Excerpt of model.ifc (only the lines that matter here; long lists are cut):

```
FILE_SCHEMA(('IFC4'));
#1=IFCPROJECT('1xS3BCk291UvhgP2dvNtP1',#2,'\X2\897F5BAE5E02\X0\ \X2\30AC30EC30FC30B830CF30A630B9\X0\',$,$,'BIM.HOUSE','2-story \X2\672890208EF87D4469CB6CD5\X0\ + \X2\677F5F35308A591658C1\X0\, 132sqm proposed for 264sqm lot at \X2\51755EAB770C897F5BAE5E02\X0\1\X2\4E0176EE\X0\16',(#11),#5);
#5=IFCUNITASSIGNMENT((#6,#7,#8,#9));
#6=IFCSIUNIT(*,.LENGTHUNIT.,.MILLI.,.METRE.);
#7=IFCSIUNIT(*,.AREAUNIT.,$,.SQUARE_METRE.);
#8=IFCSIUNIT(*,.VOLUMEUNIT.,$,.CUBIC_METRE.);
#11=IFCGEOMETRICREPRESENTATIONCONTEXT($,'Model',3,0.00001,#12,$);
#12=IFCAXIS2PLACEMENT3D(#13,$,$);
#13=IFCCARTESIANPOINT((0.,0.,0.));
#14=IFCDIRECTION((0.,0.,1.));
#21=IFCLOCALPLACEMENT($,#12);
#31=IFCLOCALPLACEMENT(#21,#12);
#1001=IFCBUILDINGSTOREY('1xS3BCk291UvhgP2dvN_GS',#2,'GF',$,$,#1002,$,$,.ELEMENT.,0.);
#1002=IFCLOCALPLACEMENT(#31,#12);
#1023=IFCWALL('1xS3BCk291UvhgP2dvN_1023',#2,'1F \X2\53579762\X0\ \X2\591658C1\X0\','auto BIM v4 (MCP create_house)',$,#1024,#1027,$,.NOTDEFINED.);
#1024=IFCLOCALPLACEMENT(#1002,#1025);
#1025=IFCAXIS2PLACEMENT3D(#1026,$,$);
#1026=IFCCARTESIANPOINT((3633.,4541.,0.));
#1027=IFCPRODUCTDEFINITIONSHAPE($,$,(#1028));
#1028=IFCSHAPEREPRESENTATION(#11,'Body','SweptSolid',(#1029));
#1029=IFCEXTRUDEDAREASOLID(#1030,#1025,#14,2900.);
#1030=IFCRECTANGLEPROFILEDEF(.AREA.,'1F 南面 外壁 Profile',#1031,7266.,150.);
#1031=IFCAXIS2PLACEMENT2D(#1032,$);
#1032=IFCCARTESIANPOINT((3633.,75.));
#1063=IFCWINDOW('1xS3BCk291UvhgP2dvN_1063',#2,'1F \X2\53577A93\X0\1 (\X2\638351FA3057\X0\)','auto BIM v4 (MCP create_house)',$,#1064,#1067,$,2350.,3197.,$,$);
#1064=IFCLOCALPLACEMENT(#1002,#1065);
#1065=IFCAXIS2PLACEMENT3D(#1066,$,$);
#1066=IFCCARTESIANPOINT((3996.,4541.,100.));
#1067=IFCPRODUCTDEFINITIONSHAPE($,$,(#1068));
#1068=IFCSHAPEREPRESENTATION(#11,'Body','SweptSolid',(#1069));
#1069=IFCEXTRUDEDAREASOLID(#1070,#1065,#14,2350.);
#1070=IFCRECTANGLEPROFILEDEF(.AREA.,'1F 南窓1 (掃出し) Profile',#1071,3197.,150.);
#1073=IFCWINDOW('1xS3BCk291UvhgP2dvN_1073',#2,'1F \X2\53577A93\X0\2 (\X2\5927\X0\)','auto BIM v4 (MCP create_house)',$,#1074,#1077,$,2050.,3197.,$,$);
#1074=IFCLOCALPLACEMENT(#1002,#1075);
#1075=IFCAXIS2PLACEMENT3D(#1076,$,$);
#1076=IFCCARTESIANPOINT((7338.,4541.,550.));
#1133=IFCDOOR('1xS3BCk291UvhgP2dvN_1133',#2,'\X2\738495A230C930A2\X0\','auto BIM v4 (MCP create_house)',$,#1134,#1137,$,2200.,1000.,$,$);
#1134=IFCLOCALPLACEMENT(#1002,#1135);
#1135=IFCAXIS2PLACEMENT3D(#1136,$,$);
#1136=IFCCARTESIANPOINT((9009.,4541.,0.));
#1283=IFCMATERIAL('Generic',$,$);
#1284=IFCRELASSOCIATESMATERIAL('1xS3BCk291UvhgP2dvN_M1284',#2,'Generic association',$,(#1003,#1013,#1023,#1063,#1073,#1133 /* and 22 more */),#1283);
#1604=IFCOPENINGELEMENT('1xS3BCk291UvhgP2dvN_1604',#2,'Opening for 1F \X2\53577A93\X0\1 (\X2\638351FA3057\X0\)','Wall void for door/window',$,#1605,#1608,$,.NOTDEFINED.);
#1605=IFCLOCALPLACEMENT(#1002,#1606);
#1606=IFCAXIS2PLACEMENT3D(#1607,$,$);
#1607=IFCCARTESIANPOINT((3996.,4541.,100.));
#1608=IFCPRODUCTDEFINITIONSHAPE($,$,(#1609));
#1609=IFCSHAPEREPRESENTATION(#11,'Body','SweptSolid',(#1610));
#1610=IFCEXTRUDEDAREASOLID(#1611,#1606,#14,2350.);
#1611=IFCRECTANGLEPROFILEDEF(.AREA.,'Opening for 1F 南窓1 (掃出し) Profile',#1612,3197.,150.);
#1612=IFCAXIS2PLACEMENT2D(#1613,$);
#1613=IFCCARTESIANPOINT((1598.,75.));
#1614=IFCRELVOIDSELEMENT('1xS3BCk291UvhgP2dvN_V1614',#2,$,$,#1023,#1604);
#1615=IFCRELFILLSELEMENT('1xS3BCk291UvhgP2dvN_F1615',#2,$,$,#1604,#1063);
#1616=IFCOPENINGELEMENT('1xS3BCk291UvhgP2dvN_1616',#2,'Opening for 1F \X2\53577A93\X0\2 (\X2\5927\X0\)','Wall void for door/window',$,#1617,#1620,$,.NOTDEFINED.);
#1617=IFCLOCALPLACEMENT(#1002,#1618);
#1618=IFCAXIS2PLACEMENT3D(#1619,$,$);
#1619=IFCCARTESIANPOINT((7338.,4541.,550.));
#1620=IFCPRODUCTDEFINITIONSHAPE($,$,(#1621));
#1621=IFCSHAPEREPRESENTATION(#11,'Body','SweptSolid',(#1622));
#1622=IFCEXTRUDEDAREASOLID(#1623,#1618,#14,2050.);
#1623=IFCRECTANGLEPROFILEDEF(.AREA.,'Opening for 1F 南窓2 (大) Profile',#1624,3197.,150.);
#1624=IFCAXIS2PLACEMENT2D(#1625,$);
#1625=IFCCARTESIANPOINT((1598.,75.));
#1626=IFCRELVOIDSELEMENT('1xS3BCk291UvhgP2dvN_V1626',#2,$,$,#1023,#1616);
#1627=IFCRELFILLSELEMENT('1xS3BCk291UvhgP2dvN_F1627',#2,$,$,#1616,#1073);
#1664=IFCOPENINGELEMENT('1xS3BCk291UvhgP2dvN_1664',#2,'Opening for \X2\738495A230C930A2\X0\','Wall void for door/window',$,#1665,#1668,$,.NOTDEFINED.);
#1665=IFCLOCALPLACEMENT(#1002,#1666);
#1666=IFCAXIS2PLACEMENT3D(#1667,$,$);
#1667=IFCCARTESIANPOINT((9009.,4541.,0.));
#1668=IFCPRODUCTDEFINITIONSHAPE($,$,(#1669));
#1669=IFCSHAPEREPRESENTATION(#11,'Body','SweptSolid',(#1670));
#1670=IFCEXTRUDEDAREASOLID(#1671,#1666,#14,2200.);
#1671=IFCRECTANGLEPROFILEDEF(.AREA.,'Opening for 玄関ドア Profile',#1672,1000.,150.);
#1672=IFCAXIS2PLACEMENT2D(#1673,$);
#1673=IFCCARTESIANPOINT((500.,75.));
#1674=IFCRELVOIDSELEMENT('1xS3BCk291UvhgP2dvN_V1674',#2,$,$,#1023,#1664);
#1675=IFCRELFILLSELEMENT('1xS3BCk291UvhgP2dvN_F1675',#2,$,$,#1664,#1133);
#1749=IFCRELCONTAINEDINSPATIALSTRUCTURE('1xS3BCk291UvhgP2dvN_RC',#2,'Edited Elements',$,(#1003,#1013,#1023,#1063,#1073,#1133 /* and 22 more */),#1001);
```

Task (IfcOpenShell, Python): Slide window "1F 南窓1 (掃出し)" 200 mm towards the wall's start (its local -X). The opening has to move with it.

```python
import ifcopenshell
import ifcopenshell.api.geometry
import ifcopenshell.util.placement
import ifcopenshell.util.unit

model = ifcopenshell.open("model.ifc")
unit_scale = ifcopenshell.util.unit.calculate_unit_scale(model)

window = model.by_id(1063)
opening = window.FillsVoids[0].RelatingOpeningElement
wall = opening.VoidsElements[0].RelatingBuildingElement

wall_matrix = ifcopenshell.util.placement.get_local_placement(wall.ObjectPlacement)
shift = wall_matrix[:3, 0] * -0.2 / unit_scale
before = ifcopenshell.util.placement.get_local_placement(window.ObjectPlacement)[:3, 3].copy()

# The window is not placed relative to its opening, so move both.
for product in (opening, window):
    matrix = ifcopenshell.util.placement.get_local_placement(product.ObjectPlacement)
    matrix[:3, 3] += shift
    ifcopenshell.api.geometry.edit_object_placement(model, product=product, matrix=matrix, is_si=False)

after = ifcopenshell.util.placement.get_local_placement(window.ObjectPlacement)[:3, 3]
print("window moved by", (after - before).round(3) + 0.0)

model.write("model_edited.ifc")
```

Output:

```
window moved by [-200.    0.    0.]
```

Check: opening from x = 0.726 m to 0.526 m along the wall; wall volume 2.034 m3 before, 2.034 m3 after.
